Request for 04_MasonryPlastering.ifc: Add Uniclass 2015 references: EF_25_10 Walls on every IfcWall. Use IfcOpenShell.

First a look at what the model holds.

```python
import ifcopenshell

model = ifcopenshell.open("04_MasonryPlastering.ifc")
print(model.schema)
print("classifications:", [c.Name for c in model.by_type("IfcClassification")])
for ifc_class in ("IfcDoor", "IfcRoof", "IfcStair", "IfcWall", "IfcWindow"):
    print(ifc_class, len(model.by_type(ifc_class)))
```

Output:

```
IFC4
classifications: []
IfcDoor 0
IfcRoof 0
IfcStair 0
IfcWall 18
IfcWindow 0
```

```python
import ifcopenshell
import ifcopenshell.api.classification

model = ifcopenshell.open("04_MasonryPlastering.ifc")

system = ifcopenshell.api.classification.add_classification(model, classification="Uniclass 2015")

codes = {
    "IfcWall": ("EF_25_10", "Walls"),
}
for ifc_class, (code, name) in codes.items():
    products = model.by_type(ifc_class)
    ifcopenshell.api.classification.add_reference(
        model, products=products, classification=system, identification=code, name=name
    )
    print(code, len(products))

model.write("04_MasonryPlastering_updated.ifc")
```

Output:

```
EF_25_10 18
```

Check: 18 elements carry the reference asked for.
